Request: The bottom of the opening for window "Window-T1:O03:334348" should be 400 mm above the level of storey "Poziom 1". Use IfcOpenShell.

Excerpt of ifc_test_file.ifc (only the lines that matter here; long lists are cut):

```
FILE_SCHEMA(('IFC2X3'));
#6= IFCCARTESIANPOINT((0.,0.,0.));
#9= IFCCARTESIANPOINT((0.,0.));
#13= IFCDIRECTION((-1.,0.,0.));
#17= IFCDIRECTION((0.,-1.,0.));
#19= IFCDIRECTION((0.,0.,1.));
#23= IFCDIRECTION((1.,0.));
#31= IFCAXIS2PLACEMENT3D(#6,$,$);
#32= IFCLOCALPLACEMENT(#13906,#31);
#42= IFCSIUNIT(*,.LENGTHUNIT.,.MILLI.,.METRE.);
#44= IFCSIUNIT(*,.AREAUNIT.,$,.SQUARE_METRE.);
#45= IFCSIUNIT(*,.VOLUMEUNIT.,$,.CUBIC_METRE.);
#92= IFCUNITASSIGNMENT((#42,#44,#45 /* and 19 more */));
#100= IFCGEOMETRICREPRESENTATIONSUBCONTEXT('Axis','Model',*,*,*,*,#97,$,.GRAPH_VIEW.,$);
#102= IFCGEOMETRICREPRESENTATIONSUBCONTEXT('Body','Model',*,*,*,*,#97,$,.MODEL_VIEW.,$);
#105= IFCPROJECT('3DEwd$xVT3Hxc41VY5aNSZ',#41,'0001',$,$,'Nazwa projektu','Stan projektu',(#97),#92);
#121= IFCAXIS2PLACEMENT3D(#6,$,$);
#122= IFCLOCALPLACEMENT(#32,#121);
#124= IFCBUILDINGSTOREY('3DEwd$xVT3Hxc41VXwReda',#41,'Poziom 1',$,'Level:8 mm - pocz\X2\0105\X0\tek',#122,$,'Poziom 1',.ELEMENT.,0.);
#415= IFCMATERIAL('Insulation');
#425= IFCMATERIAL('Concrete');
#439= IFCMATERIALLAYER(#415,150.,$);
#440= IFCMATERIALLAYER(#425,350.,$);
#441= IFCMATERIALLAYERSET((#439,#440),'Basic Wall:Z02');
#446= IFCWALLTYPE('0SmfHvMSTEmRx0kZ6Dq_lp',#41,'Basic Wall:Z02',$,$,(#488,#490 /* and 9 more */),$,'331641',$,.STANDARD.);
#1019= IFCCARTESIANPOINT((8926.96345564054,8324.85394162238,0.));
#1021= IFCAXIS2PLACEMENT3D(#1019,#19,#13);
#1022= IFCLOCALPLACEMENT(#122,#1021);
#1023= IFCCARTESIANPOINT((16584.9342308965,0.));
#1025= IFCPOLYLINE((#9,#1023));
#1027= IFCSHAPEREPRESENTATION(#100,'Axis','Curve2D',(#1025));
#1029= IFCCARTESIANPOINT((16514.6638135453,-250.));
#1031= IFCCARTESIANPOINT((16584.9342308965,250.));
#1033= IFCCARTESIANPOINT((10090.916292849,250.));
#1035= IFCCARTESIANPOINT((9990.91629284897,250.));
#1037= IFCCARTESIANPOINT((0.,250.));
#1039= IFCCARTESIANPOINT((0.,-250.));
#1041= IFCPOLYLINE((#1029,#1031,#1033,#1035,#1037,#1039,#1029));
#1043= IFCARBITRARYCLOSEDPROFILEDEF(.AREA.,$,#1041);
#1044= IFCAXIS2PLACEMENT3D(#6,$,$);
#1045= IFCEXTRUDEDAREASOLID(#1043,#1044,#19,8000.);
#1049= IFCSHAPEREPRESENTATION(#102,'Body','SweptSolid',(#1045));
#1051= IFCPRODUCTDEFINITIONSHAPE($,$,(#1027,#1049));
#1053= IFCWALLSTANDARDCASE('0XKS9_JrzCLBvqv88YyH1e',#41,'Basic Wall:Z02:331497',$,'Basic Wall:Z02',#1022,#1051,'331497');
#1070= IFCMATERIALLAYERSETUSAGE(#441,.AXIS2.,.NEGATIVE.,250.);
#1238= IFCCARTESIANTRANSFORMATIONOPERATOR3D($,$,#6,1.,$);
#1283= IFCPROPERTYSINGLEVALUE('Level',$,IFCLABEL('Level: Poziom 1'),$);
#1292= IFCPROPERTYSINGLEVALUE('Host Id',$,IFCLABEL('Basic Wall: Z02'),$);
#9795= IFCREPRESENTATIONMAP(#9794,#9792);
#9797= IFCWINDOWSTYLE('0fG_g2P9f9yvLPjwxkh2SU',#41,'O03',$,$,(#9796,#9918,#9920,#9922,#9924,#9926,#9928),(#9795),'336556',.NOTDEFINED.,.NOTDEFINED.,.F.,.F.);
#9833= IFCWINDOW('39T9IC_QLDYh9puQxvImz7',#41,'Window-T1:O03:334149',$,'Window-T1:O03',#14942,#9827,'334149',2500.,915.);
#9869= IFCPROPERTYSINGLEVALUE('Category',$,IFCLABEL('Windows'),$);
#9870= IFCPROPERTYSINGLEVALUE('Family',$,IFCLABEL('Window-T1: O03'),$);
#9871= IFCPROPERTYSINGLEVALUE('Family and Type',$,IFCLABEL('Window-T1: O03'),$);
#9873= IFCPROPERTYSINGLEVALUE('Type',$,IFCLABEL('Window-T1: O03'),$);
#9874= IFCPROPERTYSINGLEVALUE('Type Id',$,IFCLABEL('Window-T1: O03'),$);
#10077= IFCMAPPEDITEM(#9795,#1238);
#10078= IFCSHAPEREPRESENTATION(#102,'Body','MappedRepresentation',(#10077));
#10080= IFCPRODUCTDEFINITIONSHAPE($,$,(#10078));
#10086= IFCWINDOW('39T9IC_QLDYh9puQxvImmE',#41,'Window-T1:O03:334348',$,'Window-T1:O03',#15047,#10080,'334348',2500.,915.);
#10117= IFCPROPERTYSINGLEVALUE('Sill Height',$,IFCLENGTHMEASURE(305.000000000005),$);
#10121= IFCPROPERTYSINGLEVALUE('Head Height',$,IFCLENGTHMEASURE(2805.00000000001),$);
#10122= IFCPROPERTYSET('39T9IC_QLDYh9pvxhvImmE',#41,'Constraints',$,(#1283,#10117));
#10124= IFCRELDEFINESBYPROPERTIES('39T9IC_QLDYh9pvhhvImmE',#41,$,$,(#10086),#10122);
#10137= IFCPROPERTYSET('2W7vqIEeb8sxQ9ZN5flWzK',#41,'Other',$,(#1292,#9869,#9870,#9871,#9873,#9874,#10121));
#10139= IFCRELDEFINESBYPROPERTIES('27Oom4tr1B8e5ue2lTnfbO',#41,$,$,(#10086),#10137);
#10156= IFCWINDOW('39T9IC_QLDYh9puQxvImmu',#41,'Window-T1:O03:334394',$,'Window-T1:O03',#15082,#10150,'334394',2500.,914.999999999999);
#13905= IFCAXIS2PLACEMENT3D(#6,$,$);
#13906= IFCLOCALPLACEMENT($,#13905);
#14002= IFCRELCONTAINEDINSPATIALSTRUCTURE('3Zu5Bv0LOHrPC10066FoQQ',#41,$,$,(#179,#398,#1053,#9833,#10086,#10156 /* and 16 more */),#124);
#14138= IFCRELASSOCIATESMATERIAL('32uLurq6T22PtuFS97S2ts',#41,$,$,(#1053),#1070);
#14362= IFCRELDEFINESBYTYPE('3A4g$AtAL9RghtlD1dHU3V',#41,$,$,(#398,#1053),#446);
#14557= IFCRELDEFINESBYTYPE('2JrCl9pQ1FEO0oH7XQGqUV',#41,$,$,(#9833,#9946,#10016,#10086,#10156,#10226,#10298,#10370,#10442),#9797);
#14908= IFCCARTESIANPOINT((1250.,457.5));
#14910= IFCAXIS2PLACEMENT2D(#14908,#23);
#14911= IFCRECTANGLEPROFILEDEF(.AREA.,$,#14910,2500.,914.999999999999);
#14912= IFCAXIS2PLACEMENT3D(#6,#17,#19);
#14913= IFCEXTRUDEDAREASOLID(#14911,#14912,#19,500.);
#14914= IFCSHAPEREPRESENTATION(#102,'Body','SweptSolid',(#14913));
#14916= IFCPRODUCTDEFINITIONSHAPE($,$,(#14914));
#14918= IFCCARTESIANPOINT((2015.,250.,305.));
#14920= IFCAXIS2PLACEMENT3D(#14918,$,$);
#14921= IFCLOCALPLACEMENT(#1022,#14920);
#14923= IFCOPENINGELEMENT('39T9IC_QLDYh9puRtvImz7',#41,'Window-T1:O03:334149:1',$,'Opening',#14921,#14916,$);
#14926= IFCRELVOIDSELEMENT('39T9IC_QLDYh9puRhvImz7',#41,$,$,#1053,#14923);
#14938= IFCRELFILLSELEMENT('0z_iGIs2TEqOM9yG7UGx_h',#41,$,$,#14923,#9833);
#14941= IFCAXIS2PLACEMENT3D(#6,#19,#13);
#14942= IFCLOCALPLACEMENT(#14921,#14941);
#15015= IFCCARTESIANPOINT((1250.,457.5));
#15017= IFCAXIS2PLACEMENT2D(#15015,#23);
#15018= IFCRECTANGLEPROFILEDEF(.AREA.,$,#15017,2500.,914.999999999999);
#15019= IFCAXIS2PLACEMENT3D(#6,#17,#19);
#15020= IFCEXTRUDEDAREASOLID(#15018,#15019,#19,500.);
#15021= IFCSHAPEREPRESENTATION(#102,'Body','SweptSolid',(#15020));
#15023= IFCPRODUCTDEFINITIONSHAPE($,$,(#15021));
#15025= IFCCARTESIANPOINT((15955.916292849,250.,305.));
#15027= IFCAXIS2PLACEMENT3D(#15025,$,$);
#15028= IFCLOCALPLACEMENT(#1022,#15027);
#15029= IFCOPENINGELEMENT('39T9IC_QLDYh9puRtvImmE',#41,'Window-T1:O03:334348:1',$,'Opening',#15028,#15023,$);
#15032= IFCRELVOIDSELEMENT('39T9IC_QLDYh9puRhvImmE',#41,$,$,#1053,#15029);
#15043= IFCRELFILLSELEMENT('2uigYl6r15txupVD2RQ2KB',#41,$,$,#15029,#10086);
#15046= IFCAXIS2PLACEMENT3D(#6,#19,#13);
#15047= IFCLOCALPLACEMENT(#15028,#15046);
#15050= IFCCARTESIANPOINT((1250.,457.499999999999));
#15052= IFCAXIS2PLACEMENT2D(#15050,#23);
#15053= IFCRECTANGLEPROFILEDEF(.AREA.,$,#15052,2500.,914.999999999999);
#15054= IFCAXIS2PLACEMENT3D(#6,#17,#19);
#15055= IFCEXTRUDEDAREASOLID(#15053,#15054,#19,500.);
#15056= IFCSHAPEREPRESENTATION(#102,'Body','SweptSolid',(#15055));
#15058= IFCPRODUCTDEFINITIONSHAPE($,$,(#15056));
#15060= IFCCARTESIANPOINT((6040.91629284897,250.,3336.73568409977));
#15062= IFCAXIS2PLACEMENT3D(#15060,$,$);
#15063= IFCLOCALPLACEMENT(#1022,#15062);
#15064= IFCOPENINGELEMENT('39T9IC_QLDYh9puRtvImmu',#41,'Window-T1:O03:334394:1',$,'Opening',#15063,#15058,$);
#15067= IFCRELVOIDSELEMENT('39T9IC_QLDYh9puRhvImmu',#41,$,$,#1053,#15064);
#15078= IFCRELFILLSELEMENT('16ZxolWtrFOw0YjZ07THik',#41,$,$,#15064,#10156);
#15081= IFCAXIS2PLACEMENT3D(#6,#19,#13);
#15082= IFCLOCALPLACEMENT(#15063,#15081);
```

```python
import numpy as np
import ifcopenshell
import ifcopenshell.api.geometry
import ifcopenshell.api.pset
import ifcopenshell.geom
import ifcopenshell.util.element
import ifcopenshell.util.placement
import ifcopenshell.util.shape
import ifcopenshell.util.unit

model = ifcopenshell.open("ifc_test_file.ifc")
unit_scale = ifcopenshell.util.unit.calculate_unit_scale(model)

window = model.by_guid("39T9IC_QLDYh9puQxvImmE")
opening = window.FillsVoids[0].RelatingOpeningElement
storey = ifcopenshell.util.element.get_container(window, ifc_class="IfcBuildingStorey")
level = ifcopenshell.util.placement.get_local_placement(storey.ObjectPlacement)[2, 3]

# The opening's origin need not be at the sill, so measure its lowest point.
shape = ifcopenshell.geom.create_shape(ifcopenshell.geom.settings(), opening)
bottom = ifcopenshell.util.shape.get_shape_bottom_elevation(shape, shape.geometry) / unit_scale
dz = level + 0.4 / unit_scale - bottom

shift = np.array([0.0, 0.0, dz])
# The window is placed relative to its opening, so it follows when the opening moves.
matrix = ifcopenshell.util.placement.get_local_placement(opening.ObjectPlacement)
matrix[:3, 3] += shift
ifcopenshell.api.geometry.edit_object_placement(
    model, product=opening, matrix=matrix, is_si=False, should_transform_children=True
)

# Keep the stored heights in step.
pset = model.by_id(ifcopenshell.util.element.get_pset(window, "Constraints", should_inherit=False)["id"])
ifcopenshell.api.pset.edit_pset(model, pset=pset, properties={
    "Sill Height": model.create_entity("IfcLengthMeasure", ifcopenshell.util.element.get_pset(window, "Constraints", "Sill Height") + dz),
})
pset = model.by_id(ifcopenshell.util.element.get_pset(window, "Other", should_inherit=False)["id"])
ifcopenshell.api.pset.edit_pset(model, pset=pset, properties={
    "Head Height": model.create_entity("IfcLengthMeasure", ifcopenshell.util.element.get_pset(window, "Other", "Head Height") + dz),
})

print(f"moved by {dz * unit_scale:+.3f} m")

model.write("ifc_test_file_rev.ifc")
```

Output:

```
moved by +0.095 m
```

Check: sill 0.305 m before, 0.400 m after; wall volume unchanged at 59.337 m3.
